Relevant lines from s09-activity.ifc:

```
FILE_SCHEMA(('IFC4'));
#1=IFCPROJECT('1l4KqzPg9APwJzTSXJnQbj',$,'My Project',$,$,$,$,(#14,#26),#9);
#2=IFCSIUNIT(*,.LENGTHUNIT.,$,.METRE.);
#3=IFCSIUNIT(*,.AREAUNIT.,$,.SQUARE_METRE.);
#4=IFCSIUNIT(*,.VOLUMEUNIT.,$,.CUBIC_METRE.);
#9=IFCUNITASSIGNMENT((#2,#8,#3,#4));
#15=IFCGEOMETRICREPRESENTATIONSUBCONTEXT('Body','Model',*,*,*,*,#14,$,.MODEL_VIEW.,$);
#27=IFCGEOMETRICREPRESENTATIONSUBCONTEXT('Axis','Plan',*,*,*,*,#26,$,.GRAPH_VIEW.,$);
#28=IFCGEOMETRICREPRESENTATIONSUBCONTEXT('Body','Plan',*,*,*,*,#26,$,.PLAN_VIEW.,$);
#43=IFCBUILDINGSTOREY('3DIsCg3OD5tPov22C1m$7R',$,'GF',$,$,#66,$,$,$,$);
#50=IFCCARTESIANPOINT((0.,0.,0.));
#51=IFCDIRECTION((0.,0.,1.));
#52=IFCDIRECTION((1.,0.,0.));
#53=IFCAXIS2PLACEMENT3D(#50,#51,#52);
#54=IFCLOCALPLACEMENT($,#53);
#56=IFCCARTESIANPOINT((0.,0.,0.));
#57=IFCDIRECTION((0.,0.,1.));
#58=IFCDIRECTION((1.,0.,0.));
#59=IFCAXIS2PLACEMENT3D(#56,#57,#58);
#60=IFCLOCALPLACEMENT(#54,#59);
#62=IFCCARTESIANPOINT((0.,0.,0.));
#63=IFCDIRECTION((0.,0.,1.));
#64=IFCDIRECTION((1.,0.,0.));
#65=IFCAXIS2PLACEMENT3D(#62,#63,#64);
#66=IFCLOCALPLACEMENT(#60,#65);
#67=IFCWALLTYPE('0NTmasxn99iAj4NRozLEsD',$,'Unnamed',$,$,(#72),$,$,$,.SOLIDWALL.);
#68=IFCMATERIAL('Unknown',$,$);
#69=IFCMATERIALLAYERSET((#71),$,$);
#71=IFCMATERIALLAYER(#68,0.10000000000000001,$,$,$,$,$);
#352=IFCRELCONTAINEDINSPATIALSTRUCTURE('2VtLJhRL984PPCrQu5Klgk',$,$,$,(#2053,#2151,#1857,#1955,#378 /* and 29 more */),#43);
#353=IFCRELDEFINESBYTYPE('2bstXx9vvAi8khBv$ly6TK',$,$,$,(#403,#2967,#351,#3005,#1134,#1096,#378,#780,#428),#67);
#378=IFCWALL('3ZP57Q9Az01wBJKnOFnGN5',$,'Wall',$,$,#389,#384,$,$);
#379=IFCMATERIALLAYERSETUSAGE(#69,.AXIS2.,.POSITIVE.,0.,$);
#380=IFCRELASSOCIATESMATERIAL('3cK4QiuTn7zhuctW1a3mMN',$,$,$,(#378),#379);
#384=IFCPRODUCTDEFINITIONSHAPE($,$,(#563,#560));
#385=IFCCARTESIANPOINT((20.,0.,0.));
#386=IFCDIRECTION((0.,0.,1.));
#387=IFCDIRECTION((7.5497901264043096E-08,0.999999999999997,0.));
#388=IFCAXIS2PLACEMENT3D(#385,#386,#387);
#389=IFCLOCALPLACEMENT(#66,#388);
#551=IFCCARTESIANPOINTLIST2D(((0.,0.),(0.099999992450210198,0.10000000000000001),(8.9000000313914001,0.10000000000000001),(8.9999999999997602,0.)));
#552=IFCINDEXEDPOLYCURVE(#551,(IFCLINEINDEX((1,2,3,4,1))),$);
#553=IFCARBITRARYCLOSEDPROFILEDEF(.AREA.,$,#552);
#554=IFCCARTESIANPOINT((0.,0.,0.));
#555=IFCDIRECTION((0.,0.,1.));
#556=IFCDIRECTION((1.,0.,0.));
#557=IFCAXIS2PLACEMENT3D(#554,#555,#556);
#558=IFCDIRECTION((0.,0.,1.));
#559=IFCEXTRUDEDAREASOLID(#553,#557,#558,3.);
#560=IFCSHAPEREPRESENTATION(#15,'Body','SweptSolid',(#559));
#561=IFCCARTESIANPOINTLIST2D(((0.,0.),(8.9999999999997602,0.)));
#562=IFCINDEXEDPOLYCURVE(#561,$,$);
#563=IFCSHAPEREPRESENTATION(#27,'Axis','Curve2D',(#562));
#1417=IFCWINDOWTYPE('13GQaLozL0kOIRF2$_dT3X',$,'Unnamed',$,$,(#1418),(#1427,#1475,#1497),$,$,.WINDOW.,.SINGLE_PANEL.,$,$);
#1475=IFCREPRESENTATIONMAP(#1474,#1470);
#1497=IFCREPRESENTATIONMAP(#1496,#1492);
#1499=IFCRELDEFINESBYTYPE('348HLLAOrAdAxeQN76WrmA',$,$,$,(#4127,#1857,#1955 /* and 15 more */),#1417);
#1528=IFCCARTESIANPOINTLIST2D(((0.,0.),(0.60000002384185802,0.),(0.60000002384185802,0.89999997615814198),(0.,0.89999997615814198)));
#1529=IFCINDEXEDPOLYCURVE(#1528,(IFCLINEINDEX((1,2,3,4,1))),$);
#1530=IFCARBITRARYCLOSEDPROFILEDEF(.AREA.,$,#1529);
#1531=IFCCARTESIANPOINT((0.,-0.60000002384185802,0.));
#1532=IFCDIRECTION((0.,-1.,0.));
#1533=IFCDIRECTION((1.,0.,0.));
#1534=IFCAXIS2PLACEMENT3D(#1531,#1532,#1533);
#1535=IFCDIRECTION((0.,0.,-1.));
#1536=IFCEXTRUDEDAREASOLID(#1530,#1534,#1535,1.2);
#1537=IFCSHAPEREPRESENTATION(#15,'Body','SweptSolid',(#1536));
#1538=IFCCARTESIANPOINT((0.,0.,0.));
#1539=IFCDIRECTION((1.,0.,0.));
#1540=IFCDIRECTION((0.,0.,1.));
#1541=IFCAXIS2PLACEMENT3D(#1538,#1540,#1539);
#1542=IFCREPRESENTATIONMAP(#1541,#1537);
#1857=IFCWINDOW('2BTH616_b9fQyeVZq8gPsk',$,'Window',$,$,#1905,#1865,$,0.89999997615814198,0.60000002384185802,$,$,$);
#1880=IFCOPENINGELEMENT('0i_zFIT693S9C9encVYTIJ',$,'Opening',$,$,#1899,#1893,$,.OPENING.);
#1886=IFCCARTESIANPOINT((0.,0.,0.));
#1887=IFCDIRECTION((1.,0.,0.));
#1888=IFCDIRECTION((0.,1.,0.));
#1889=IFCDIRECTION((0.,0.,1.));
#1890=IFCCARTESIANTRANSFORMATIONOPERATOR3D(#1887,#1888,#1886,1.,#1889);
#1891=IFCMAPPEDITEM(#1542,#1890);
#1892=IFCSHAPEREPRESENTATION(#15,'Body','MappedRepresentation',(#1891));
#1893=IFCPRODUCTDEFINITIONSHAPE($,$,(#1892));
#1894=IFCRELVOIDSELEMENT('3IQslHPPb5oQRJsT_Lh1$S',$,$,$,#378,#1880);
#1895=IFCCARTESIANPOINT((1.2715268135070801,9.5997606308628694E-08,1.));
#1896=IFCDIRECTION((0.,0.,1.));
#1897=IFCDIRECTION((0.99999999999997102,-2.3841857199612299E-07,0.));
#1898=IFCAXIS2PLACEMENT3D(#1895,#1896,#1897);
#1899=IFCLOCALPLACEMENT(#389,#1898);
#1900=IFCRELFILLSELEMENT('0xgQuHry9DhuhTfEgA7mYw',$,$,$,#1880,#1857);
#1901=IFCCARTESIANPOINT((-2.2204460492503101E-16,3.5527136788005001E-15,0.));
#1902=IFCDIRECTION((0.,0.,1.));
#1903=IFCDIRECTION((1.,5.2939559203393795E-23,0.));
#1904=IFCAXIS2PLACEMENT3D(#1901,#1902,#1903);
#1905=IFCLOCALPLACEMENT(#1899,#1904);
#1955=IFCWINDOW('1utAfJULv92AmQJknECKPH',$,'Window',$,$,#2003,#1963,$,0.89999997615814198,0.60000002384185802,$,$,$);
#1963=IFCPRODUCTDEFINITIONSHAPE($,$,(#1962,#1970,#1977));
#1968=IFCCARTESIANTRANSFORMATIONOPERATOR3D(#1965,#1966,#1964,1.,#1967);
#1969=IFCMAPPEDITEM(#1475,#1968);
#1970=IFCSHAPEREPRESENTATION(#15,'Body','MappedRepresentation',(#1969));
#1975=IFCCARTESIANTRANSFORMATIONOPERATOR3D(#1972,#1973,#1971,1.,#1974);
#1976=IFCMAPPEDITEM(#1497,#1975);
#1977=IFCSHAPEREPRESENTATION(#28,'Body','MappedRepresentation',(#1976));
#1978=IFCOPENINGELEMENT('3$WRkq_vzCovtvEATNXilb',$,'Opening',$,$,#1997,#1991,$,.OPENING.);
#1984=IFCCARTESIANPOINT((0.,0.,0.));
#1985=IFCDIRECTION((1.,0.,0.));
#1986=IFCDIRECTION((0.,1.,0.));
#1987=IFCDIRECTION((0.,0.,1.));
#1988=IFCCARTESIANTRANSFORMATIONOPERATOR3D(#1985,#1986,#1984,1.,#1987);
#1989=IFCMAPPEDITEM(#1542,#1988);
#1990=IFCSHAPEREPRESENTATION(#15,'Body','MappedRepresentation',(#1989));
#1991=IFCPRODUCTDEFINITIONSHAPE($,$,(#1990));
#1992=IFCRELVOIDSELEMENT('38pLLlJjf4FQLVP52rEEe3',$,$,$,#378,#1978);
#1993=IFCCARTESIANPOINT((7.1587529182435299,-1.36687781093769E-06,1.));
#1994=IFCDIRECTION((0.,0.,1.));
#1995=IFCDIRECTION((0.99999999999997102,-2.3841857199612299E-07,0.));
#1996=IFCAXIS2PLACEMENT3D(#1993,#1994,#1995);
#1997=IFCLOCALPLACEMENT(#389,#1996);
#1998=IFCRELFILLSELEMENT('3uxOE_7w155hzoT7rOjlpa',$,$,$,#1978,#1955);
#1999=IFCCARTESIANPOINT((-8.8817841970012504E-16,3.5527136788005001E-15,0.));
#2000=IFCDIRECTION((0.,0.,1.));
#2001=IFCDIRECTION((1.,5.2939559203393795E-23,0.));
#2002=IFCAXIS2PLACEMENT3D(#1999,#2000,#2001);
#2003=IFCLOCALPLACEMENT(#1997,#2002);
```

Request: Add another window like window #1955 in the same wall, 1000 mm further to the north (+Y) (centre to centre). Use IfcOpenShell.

```python
import ifcopenshell
import ifcopenshell.api.feature
import ifcopenshell.api.geometry
import ifcopenshell.api.root
import ifcopenshell.geom
import ifcopenshell.util.element
import ifcopenshell.util.placement
import ifcopenshell.util.shape
import ifcopenshell.util.unit

model = ifcopenshell.open("s09-activity.ifc")
unit_scale = ifcopenshell.util.unit.calculate_unit_scale(model)
settings = ifcopenshell.geom.settings()


def volume(element):
    """Net volume in cubic metres, openings subtracted."""
    shape = ifcopenshell.geom.create_shape(settings, element)
    return ifcopenshell.util.shape.get_volume(shape.geometry)


window = model.by_guid("1utAfJULv92AmQJknECKPH")
opening = window.FillsVoids[0].RelatingOpeningElement
wall = opening.VoidsElements[0].RelatingBuildingElement
before = volume(wall)
shift = ifcopenshell.util.placement.get_local_placement(wall.ObjectPlacement)[:3, 0] * 1 / unit_scale

# copy_class copies the void relationship, type, container and properties, but no geometry.
new_opening = ifcopenshell.api.root.copy_class(model, product=opening)
new_opening.Representation = ifcopenshell.util.element.copy_deep(
    model, opening.Representation, exclude=["IfcGeometricRepresentationContext", "IfcRepresentationMap"]
)
new_window = ifcopenshell.api.root.copy_class(model, product=window)
new_window.Representation = ifcopenshell.util.element.copy_deep(
    model, window.Representation, exclude=["IfcGeometricRepresentationContext", "IfcRepresentationMap"]
)
ifcopenshell.api.feature.add_filling(model, opening=new_opening, element=new_window)

for old, new in ((opening, new_opening), (window, new_window)):
    matrix = ifcopenshell.util.placement.get_local_placement(old.ObjectPlacement)
    matrix[:3, 3] += shift
    ifcopenshell.api.geometry.edit_object_placement(model, product=new, matrix=matrix, is_si=False)

after = volume(wall)

print(f"wall volume {before:.3f} -> {after:.3f} m3")

model.write("s09-activity-out.ifc")
```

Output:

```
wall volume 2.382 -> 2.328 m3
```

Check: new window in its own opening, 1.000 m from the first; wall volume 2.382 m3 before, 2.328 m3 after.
